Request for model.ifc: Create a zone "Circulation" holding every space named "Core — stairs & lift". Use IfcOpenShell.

First a look at what the model holds.

```python
import ifcopenshell

model = ifcopenshell.open("model.ifc")
print(model.schema)
seen = {}
for space in model.by_type("IfcSpace"):
    seen[space.Name] = seen.get(space.Name, 0) + 1
for name, count in sorted(seen.items(), key=str):
    print(count, "x", name)
print("zones:", [z.Name for z in model.by_type("IfcZone")][:20])
```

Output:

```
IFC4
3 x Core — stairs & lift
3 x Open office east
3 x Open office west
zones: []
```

```python
import ifcopenshell
import ifcopenshell.api.group
import ifcopenshell.api.root

model = ifcopenshell.open("model.ifc")

names = {"Core — stairs & lift"}
spaces = [s for s in model.by_type("IfcSpace") if s.Name in names]

zone = ifcopenshell.api.root.create_entity(model, ifc_class="IfcZone", name="Circulation")
ifcopenshell.api.group.assign_group(model, products=spaces, group=zone)
print(len(spaces), "spaces in", zone.Name)

model.write("model-out.ifc")
```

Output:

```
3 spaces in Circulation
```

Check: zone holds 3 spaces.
